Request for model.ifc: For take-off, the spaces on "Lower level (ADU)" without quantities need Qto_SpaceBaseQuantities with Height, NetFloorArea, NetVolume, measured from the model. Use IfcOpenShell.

First a look at what the model holds.

```python
import ifcopenshell
import ifcopenshell.util.element
import ifcopenshell.util.unit

model = ifcopenshell.open("model.ifc")
print(model.schema)
for unit_type in ("LENGTHUNIT", "AREAUNIT", "VOLUMEUNIT"):
    print(unit_type, ifcopenshell.util.unit.calculate_unit_scale(model, unit_type))
storey = next(s for s in model.by_type("IfcBuildingStorey") if s.Name == "Lower level (ADU)")
spaces = [e for e in ifcopenshell.util.element.get_decomposition(storey) if e.is_a("IfcSpace")]
for e in sorted(spaces, key=lambda e: e.id()):
    print(e.id(), e.is_a(), e.Name, list(ifcopenshell.util.element.get_psets(e, qtos_only=True)), sep=" | ")
```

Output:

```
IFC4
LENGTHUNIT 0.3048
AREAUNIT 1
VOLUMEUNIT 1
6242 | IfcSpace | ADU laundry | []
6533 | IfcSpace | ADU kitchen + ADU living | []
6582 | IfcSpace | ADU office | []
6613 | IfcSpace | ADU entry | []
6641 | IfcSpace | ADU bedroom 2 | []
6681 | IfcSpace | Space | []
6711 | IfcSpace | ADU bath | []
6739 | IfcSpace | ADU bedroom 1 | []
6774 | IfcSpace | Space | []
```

```python
import ifcopenshell
import ifcopenshell.api.pset
import ifcopenshell.geom
import ifcopenshell.util.element
import ifcopenshell.util.shape
import ifcopenshell.util.unit

model = ifcopenshell.open("model.ifc")
unit_scale = ifcopenshell.util.unit.calculate_unit_scale(model)
area_scale = ifcopenshell.util.unit.calculate_unit_scale(model, "AREAUNIT")
volume_scale = ifcopenshell.util.unit.calculate_unit_scale(model, "VOLUMEUNIT")
settings = ifcopenshell.geom.settings()

storey = next(s for s in model.by_type("IfcBuildingStorey") if s.Name == "Lower level (ADU)")
spaces = [e for e in ifcopenshell.util.element.get_decomposition(storey) if e.is_a("IfcSpace")]

for e in sorted(spaces, key=lambda e: e.id()):
    if ifcopenshell.util.element.get_psets(e, qtos_only=True, should_inherit=False):
        continue
    # Geometry comes back in metres, in the element's own axes.
    shape = ifcopenshell.geom.create_shape(settings, e)
    values = {
        "Height": ifcopenshell.util.shape.get_z(shape.geometry) / unit_scale,
        "NetFloorArea": ifcopenshell.util.shape.get_footprint_area(shape.geometry) / area_scale,
        "NetVolume": ifcopenshell.util.shape.get_volume(shape.geometry) / volume_scale,
    }
    qto = ifcopenshell.api.pset.add_qto(model, product=e, name="Qto_SpaceBaseQuantities")
    ifcopenshell.api.pset.edit_qto(model, qto=qto, properties=values)
    print(e.id(), {k: round(v, 3) for k, v in values.items()})

model.write("model_edited.ifc")
```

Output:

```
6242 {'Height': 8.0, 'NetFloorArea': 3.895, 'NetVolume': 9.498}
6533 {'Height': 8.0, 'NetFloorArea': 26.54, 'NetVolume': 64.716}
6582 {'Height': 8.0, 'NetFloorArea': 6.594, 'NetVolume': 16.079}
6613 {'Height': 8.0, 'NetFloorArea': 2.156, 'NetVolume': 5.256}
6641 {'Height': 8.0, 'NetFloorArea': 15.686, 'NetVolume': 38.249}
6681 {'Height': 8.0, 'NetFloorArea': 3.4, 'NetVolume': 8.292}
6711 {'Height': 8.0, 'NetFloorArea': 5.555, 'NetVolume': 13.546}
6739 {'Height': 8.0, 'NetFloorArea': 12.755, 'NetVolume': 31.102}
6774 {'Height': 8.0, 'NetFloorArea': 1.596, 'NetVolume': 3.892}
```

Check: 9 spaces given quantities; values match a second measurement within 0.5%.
